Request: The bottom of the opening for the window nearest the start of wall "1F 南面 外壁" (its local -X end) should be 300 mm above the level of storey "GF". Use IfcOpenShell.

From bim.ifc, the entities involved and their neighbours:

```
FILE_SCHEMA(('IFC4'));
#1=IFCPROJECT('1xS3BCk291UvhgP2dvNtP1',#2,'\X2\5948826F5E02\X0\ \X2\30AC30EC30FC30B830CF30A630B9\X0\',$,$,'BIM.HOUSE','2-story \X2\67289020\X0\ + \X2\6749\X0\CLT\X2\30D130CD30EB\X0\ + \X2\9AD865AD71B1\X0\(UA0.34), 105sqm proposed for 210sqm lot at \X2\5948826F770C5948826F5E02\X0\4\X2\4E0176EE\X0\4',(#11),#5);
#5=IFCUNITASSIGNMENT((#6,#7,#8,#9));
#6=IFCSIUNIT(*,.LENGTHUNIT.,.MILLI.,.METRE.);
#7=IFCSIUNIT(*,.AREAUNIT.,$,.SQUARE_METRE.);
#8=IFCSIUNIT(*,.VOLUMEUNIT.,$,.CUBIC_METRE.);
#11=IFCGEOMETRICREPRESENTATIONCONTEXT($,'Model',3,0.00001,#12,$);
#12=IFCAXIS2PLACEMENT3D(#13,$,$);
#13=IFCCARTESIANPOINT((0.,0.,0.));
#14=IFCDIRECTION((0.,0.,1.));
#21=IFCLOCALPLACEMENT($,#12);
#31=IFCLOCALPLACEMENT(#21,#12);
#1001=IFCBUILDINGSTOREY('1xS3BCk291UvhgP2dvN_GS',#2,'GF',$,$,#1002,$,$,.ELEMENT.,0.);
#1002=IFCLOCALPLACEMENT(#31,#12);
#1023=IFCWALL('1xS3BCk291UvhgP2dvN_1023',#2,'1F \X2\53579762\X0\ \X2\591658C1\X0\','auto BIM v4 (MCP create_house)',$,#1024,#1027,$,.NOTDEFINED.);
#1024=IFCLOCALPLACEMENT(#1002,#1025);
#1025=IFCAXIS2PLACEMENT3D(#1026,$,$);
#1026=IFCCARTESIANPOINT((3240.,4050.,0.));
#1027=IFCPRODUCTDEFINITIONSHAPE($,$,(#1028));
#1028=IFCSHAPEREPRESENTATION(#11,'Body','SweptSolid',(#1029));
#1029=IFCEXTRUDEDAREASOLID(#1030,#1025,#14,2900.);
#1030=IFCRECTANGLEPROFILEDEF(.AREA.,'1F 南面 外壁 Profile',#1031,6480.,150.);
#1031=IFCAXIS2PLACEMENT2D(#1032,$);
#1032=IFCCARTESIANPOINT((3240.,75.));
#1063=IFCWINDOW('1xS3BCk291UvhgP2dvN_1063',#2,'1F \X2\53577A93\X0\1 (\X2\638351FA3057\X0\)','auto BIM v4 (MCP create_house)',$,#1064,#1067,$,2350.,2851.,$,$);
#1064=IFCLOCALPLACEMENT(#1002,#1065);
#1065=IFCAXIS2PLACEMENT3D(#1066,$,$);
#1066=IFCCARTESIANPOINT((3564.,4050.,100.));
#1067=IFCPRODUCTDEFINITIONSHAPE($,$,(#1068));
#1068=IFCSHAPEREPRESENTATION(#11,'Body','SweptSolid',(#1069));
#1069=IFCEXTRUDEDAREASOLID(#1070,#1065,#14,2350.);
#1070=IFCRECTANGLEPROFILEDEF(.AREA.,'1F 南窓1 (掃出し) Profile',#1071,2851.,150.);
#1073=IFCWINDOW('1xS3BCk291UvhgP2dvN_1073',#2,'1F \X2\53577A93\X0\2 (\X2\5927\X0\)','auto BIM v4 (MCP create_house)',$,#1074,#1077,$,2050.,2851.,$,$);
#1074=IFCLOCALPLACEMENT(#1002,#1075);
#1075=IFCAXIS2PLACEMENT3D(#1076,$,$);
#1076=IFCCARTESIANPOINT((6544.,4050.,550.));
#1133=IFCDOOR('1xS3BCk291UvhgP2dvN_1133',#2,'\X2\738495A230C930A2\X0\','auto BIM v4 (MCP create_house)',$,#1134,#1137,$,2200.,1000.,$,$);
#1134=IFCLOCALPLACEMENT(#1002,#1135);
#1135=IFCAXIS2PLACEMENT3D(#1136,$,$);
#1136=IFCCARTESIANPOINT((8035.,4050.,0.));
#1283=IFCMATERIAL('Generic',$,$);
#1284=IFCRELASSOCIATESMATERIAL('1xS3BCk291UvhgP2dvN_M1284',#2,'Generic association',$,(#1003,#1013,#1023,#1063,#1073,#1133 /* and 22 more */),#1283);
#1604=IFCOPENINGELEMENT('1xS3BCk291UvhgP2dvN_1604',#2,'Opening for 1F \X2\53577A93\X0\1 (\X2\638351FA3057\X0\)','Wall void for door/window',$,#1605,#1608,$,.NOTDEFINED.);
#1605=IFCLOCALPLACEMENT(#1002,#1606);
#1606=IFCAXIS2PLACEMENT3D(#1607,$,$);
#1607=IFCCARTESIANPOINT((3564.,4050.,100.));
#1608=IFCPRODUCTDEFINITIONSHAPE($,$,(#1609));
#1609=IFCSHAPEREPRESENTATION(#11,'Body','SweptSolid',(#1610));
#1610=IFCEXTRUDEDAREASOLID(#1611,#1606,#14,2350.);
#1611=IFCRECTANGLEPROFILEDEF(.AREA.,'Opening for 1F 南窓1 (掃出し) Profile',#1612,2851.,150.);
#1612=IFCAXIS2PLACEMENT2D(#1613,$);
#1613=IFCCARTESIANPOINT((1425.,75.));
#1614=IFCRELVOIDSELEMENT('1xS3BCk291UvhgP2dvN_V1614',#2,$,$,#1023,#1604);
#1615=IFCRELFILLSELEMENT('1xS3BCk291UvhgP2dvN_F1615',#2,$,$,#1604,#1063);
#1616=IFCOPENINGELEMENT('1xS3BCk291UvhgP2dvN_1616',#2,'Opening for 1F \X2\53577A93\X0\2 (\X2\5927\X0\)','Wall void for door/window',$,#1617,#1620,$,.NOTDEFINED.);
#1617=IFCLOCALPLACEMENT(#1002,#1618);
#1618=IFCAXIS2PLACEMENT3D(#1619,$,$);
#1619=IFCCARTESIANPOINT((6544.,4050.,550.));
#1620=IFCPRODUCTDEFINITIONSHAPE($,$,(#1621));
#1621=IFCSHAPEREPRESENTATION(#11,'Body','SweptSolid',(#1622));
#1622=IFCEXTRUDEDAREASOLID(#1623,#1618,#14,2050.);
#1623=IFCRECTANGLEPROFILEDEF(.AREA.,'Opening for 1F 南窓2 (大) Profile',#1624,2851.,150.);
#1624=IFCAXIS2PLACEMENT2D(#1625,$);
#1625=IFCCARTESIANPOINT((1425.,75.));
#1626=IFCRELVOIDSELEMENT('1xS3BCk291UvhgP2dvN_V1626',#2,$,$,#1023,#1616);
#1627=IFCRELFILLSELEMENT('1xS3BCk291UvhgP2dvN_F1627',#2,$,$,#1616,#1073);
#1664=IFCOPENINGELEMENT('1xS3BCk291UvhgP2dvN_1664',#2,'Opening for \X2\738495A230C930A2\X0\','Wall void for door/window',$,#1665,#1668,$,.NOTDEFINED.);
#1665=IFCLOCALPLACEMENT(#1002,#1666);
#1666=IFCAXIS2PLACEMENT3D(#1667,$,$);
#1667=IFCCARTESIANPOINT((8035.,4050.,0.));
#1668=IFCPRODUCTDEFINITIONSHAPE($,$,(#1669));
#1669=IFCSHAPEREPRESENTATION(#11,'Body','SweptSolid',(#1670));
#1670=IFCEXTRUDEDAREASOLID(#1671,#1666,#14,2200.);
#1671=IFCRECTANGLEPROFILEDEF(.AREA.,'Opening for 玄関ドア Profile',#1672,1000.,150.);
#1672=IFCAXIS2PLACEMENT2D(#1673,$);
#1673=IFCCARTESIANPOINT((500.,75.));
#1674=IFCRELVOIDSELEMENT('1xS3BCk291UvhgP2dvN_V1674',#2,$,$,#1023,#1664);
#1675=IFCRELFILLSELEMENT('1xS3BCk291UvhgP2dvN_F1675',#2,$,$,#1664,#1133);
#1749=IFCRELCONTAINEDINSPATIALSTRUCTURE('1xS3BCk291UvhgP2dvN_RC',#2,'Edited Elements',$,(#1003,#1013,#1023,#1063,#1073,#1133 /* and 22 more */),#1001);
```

```python
import numpy as np
import ifcopenshell
import ifcopenshell.api.geometry
import ifcopenshell.geom
import ifcopenshell.util.element
import ifcopenshell.util.placement
import ifcopenshell.util.shape
import ifcopenshell.util.unit

model = ifcopenshell.open("bim.ifc")
unit_scale = ifcopenshell.util.unit.calculate_unit_scale(model)

window = model.by_guid("1xS3BCk291UvhgP2dvN_1063")
opening = window.FillsVoids[0].RelatingOpeningElement
storey = ifcopenshell.util.element.get_container(window, ifc_class="IfcBuildingStorey")
level = ifcopenshell.util.placement.get_local_placement(storey.ObjectPlacement)[2, 3]

# The opening's origin need not be at the sill, so measure its lowest point.
shape = ifcopenshell.geom.create_shape(ifcopenshell.geom.settings(), opening)
bottom = ifcopenshell.util.shape.get_shape_bottom_elevation(shape, shape.geometry) / unit_scale
dz = level + 300.0 - bottom

shift = np.array([0.0, 0.0, dz])
# The window is not placed relative to its opening, so move both.
for product in (opening, window):
    matrix = ifcopenshell.util.placement.get_local_placement(product.ObjectPlacement)
    matrix[:3, 3] += shift
    ifcopenshell.api.geometry.edit_object_placement(model, product=product, matrix=matrix, is_si=False)

print(f"moved by {dz * unit_scale:+.3f} m")

model.write("bim_rev.ifc")
```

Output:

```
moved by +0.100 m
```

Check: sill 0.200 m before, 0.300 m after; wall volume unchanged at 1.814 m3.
